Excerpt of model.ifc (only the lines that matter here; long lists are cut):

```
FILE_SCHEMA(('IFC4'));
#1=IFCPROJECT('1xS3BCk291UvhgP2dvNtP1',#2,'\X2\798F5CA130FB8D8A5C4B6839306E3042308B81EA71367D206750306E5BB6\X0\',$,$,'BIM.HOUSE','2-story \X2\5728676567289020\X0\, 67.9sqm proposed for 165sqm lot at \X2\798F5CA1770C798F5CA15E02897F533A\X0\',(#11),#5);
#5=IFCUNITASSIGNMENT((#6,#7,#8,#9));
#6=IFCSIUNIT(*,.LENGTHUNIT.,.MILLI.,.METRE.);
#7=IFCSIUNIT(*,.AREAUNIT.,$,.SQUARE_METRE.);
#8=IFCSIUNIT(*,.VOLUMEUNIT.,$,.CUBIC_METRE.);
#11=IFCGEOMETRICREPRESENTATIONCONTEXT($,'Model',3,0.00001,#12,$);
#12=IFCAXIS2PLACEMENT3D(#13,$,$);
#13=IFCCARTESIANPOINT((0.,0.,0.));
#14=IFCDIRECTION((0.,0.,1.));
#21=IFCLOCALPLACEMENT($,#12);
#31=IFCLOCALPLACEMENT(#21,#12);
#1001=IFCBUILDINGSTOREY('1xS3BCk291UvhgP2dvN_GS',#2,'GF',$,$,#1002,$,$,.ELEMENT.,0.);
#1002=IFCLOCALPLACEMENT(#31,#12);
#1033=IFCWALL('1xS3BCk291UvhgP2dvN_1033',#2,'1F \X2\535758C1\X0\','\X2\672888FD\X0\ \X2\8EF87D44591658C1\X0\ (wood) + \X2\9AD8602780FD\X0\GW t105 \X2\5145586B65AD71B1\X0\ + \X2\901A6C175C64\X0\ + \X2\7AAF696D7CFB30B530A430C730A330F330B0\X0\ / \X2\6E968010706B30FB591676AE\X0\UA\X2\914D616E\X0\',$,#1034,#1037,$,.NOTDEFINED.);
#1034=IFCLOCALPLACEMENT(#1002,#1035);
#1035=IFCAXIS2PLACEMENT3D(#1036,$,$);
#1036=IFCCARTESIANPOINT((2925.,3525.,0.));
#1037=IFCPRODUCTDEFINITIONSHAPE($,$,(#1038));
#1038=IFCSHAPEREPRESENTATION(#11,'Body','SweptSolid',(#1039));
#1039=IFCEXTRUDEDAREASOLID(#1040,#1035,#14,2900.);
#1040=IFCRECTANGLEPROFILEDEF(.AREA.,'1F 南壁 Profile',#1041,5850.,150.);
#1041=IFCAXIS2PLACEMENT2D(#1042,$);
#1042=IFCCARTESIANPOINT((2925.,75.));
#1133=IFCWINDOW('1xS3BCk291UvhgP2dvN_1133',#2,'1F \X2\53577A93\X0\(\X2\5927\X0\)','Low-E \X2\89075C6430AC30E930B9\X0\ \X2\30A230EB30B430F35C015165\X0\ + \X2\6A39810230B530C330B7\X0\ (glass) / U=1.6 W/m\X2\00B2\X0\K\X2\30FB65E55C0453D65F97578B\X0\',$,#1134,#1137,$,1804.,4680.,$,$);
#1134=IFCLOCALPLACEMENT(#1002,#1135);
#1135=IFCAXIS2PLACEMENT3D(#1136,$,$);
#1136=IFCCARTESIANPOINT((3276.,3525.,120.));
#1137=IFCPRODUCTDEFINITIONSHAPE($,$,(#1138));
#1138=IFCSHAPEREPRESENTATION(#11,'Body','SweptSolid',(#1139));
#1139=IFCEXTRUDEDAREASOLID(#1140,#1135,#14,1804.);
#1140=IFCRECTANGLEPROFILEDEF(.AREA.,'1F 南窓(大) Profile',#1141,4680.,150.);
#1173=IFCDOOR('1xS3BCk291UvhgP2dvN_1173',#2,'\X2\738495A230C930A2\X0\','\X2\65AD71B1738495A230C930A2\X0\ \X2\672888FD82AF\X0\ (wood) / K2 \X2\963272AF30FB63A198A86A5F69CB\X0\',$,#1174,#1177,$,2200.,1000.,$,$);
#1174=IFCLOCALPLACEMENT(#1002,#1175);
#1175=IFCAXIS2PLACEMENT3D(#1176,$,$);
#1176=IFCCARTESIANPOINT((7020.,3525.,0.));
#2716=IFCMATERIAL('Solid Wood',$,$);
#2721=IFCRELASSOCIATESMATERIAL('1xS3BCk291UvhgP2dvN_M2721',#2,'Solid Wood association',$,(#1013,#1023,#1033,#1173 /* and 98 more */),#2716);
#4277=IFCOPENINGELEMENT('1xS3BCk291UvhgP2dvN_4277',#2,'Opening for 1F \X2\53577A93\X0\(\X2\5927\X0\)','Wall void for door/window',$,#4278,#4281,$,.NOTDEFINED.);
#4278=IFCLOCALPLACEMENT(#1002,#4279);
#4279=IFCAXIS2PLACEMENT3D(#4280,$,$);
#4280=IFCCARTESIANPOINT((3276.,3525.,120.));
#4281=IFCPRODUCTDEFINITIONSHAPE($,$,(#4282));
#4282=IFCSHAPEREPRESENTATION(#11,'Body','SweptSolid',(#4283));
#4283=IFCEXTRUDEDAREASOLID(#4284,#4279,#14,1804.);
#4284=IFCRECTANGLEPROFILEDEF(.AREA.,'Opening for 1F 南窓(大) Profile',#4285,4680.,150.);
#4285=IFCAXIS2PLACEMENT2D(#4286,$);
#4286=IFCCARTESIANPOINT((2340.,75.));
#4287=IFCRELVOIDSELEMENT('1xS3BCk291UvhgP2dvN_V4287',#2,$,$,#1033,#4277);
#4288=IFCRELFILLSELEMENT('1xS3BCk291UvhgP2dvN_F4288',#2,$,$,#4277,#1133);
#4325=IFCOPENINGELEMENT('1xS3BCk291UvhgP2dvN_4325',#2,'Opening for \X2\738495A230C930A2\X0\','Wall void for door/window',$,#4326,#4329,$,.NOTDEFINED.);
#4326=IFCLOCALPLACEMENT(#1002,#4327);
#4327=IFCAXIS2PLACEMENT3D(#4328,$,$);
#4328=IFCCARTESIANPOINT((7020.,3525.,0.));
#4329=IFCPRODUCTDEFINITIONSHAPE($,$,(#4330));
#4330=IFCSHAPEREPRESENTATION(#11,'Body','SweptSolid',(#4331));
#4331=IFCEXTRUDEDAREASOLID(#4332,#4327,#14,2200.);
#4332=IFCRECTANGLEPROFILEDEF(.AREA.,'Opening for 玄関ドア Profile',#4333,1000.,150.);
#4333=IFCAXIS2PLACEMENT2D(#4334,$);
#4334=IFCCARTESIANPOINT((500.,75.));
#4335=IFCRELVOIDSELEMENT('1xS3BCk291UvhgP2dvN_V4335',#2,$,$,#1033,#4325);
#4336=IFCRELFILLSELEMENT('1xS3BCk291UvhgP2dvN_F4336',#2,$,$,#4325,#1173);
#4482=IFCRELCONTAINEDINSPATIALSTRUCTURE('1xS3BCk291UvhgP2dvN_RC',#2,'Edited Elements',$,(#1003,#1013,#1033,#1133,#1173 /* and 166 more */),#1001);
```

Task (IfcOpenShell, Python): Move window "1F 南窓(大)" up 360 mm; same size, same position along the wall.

```python
import numpy as np
import ifcopenshell
import ifcopenshell.api.geometry
import ifcopenshell.util.placement
import ifcopenshell.util.unit

model = ifcopenshell.open("model.ifc")
unit_scale = ifcopenshell.util.unit.calculate_unit_scale(model)

window = model.by_guid("1xS3BCk291UvhgP2dvN_1133")
opening = window.FillsVoids[0].RelatingOpeningElement
dz = 360.0

shift = np.array([0.0, 0.0, dz])
# The window is not placed relative to its opening, so move both.
for product in (opening, window):
    matrix = ifcopenshell.util.placement.get_local_placement(product.ObjectPlacement)
    matrix[:3, 3] += shift
    ifcopenshell.api.geometry.edit_object_placement(model, product=product, matrix=matrix, is_si=False)

print(f"moved by {dz * unit_scale:+.3f} m")

model.write("model_rev.ifc")
```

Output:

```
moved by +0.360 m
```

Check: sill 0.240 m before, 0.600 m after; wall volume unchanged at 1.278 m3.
